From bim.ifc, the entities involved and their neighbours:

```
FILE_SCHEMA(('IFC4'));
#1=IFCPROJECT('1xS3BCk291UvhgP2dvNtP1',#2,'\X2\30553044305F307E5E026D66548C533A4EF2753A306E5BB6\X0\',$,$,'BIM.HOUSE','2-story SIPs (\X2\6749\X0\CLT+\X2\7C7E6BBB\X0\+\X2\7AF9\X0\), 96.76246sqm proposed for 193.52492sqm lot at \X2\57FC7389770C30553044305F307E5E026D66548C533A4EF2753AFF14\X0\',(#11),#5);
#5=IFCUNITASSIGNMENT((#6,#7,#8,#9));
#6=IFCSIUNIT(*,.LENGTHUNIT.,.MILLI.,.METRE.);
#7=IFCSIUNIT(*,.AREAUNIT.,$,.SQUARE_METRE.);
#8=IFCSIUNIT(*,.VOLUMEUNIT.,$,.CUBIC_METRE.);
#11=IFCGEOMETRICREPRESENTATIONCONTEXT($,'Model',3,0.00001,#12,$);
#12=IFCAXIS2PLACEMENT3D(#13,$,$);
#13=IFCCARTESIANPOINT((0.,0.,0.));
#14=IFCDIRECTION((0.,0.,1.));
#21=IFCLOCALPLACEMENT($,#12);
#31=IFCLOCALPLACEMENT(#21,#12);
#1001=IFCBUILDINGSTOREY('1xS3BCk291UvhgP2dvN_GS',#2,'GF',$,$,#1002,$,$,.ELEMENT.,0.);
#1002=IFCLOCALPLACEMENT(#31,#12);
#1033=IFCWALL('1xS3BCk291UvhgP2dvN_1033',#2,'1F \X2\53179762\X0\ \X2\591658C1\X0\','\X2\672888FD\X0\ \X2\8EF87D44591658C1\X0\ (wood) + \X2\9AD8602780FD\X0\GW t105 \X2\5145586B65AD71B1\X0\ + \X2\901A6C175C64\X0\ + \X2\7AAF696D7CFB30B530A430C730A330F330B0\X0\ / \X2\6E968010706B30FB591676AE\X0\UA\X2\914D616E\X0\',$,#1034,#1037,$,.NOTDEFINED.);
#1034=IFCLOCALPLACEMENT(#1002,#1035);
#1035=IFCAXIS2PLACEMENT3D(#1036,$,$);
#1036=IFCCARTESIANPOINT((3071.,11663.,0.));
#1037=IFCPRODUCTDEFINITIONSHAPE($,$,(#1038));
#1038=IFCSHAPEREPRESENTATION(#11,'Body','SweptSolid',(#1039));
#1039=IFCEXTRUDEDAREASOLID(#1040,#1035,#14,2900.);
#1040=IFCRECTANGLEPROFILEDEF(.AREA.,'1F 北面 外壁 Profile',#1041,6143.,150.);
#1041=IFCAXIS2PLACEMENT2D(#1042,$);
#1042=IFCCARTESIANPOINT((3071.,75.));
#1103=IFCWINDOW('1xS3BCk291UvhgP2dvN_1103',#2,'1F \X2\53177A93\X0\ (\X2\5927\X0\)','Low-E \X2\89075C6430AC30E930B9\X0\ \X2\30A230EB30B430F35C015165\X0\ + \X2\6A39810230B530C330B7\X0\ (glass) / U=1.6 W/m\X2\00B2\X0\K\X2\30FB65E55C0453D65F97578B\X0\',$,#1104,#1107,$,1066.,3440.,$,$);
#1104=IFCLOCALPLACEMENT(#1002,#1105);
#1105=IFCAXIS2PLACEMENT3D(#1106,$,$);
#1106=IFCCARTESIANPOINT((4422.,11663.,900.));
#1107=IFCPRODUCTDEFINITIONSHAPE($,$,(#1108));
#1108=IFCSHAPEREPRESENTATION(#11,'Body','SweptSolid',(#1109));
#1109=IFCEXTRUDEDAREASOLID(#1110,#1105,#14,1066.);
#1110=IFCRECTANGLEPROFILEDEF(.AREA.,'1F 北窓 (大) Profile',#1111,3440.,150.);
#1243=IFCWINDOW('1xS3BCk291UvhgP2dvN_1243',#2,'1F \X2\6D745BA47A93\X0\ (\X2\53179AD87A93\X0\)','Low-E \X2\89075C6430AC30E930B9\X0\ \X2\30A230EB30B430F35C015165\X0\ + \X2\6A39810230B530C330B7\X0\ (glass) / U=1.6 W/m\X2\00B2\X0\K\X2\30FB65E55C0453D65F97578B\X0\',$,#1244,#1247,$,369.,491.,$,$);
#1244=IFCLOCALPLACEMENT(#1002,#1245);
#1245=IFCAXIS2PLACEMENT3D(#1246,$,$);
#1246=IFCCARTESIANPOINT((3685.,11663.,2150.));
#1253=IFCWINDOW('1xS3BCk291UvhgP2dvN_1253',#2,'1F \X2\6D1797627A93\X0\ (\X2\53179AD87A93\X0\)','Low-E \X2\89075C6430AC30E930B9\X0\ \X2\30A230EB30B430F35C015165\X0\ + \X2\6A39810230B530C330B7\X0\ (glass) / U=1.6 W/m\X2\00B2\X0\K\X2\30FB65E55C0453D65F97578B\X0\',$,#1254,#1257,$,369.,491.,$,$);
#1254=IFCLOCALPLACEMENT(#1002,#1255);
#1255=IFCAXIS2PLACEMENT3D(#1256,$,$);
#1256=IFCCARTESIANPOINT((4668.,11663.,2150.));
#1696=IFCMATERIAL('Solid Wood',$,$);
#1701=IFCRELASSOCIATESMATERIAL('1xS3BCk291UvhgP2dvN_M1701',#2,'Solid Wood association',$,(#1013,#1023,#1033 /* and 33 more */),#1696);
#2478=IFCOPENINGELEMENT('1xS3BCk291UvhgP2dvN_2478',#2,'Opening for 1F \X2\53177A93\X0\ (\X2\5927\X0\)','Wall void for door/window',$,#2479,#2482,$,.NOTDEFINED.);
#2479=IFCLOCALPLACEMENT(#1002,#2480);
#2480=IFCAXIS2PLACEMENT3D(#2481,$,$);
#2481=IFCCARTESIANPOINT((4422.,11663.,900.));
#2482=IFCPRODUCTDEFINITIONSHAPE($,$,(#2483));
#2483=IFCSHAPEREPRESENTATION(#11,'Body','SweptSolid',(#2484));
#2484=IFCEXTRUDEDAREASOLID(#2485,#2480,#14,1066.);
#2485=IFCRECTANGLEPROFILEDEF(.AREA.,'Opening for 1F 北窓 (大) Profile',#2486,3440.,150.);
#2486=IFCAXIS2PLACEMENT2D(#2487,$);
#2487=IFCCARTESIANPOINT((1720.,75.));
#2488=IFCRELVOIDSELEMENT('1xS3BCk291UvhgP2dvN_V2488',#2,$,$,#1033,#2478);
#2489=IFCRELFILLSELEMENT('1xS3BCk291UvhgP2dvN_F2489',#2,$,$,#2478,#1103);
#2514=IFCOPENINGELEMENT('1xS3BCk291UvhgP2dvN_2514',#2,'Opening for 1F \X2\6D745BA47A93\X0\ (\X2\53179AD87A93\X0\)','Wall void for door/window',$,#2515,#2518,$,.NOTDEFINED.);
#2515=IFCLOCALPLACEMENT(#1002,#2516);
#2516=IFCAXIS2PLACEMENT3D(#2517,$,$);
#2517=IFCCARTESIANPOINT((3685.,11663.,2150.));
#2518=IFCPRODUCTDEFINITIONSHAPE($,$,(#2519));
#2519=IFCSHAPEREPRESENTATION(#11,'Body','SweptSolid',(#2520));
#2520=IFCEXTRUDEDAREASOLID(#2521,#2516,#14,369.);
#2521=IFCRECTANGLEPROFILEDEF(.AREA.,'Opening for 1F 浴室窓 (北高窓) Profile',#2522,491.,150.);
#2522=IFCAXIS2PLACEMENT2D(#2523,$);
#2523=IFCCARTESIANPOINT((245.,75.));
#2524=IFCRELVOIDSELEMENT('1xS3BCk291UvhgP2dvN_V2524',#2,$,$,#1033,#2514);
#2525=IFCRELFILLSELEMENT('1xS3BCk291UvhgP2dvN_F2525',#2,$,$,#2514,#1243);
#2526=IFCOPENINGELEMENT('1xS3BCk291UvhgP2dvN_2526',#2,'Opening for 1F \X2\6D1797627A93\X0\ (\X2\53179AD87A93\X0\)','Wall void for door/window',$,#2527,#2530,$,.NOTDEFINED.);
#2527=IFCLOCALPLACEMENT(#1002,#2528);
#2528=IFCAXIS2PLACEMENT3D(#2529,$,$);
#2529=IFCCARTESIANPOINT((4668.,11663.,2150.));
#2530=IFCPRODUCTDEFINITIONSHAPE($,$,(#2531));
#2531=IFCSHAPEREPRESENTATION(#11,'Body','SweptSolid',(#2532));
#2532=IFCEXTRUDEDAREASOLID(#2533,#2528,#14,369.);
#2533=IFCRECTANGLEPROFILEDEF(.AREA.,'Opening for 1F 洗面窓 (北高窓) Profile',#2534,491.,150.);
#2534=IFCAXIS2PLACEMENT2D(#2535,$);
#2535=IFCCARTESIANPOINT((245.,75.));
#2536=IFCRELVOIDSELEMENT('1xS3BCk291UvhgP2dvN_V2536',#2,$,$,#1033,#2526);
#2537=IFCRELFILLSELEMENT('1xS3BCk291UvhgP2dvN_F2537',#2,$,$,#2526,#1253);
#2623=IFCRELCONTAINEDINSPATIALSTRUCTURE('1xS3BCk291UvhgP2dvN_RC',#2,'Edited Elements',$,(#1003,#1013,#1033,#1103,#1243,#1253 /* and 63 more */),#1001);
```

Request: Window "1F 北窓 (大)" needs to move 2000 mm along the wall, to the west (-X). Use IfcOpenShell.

```python
import ifcopenshell
import ifcopenshell.api.geometry
import ifcopenshell.util.placement

model = ifcopenshell.open("bim.ifc")

window = model.by_guid("1xS3BCk291UvhgP2dvN_1103")
opening = window.FillsVoids[0].RelatingOpeningElement
wall = opening.VoidsElements[0].RelatingBuildingElement

wall_matrix = ifcopenshell.util.placement.get_local_placement(wall.ObjectPlacement)
shift = wall_matrix[:3, 0] * -2000.0
before = ifcopenshell.util.placement.get_local_placement(window.ObjectPlacement)[:3, 3].copy()

# The window is not placed relative to its opening, so move both.
for product in (opening, window):
    matrix = ifcopenshell.util.placement.get_local_placement(product.ObjectPlacement)
    matrix[:3, 3] += shift
    ifcopenshell.api.geometry.edit_object_placement(model, product=product, matrix=matrix, is_si=False)

after = ifcopenshell.util.placement.get_local_placement(window.ObjectPlacement)[:3, 3]
print("window moved by", (after - before).round(3) + 0.0)

model.write("bim_v2.ifc")
```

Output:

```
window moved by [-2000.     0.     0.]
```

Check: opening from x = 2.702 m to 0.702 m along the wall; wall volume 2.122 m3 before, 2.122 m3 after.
